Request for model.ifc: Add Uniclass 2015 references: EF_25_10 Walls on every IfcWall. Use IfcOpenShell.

First a look at what the model holds.

```python
import ifcopenshell

model = ifcopenshell.open("model.ifc")
print(model.schema)
print("classifications:", [c.Name for c in model.by_type("IfcClassification")])
for ifc_class in ("IfcDoor", "IfcRoof", "IfcStair", "IfcWall", "IfcWindow"):
    print(ifc_class, len(model.by_type(ifc_class)))
```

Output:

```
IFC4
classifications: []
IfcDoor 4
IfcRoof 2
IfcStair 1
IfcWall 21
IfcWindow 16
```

```python
import ifcopenshell
import ifcopenshell.api.classification

model = ifcopenshell.open("model.ifc")

system = ifcopenshell.api.classification.add_classification(model, classification="Uniclass 2015")

codes = {
    "IfcWall": ("EF_25_10", "Walls"),
}
for ifc_class, (code, name) in codes.items():
    products = model.by_type(ifc_class)
    ifcopenshell.api.classification.add_reference(
        model, products=products, classification=system, identification=code, name=name
    )
    print(code, len(products))

model.write("model_updated.ifc")
```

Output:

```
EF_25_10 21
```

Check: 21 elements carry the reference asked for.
